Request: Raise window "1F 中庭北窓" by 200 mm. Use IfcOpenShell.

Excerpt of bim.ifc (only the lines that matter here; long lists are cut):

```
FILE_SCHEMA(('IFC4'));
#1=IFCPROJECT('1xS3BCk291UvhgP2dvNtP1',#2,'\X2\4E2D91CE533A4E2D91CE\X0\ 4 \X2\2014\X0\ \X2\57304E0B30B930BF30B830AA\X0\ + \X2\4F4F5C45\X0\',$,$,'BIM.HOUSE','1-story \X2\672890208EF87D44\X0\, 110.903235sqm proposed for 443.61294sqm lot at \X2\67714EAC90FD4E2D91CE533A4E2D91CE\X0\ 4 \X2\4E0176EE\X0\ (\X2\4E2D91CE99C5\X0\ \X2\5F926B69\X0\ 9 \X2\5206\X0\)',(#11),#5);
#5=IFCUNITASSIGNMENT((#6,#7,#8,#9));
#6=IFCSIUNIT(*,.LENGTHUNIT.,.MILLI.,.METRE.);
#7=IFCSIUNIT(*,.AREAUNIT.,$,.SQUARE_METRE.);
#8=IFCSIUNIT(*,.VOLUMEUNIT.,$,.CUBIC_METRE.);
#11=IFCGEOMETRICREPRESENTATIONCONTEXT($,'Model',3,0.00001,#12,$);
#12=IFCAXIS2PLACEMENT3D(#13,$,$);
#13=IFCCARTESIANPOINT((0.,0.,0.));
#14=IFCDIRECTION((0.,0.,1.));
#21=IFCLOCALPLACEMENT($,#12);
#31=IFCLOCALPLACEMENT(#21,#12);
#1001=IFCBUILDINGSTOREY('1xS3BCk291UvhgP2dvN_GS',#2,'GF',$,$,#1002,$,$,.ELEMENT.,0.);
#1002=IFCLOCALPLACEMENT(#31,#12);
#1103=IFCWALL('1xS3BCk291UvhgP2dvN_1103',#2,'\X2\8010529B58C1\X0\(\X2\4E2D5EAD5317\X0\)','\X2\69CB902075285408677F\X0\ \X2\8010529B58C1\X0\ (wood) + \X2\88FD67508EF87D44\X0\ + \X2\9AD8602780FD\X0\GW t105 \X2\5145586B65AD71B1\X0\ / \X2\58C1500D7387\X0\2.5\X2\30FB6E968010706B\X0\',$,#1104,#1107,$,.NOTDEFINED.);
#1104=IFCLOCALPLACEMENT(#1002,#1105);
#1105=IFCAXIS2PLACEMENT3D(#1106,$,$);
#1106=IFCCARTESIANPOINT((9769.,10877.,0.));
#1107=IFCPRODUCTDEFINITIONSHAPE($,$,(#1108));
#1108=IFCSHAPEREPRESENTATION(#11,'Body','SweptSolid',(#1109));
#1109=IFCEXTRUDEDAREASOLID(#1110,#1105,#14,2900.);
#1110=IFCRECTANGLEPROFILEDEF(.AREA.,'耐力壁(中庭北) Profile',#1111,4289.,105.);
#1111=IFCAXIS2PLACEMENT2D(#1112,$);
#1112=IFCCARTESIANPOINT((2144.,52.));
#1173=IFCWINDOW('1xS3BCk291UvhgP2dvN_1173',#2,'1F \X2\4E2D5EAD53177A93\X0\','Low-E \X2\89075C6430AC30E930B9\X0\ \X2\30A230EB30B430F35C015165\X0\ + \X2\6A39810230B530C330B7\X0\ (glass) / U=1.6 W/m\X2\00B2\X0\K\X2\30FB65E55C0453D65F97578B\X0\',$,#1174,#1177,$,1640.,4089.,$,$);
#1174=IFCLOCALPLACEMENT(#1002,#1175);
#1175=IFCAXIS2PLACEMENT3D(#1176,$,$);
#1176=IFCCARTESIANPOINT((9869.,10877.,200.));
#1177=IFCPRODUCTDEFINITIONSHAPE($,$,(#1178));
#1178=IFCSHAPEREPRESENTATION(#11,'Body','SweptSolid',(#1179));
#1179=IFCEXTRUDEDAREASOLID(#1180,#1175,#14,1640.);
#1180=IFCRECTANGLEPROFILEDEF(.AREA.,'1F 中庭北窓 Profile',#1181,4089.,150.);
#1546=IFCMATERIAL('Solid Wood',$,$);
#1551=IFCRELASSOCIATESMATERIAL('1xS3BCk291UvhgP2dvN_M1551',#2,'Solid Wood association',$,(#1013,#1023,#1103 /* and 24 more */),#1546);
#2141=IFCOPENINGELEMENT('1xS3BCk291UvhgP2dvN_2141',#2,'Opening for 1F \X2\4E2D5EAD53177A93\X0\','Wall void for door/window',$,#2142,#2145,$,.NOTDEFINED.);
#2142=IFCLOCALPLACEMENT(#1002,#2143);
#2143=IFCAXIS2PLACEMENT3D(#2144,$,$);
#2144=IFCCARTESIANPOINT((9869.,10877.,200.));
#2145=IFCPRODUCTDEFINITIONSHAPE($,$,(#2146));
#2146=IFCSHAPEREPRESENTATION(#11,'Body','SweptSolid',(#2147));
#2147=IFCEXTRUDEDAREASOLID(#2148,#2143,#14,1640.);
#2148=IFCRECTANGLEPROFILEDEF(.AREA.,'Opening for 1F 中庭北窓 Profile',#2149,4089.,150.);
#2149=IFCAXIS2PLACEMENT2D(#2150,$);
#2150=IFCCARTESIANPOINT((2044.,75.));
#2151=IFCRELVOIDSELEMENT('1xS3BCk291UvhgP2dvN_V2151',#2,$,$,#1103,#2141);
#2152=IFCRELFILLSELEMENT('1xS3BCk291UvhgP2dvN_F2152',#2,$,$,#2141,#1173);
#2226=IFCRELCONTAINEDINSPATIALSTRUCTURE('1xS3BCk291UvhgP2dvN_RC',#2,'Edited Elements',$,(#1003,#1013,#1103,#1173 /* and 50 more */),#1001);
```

```python
import numpy as np
import ifcopenshell
import ifcopenshell.api.geometry
import ifcopenshell.util.placement
import ifcopenshell.util.unit

model = ifcopenshell.open("bim.ifc")
unit_scale = ifcopenshell.util.unit.calculate_unit_scale(model)

window = model.by_guid("1xS3BCk291UvhgP2dvN_1173")
opening = window.FillsVoids[0].RelatingOpeningElement
dz = 200.0

shift = np.array([0.0, 0.0, dz])
# The window is not placed relative to its opening, so move both.
for product in (opening, window):
    matrix = ifcopenshell.util.placement.get_local_placement(product.ObjectPlacement)
    matrix[:3, 3] += shift
    ifcopenshell.api.geometry.edit_object_placement(model, product=product, matrix=matrix, is_si=False)

print(f"moved by {dz * unit_scale:+.3f} m")

model.write("bim-out.ifc")
```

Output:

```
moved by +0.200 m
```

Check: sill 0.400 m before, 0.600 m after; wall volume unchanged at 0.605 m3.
